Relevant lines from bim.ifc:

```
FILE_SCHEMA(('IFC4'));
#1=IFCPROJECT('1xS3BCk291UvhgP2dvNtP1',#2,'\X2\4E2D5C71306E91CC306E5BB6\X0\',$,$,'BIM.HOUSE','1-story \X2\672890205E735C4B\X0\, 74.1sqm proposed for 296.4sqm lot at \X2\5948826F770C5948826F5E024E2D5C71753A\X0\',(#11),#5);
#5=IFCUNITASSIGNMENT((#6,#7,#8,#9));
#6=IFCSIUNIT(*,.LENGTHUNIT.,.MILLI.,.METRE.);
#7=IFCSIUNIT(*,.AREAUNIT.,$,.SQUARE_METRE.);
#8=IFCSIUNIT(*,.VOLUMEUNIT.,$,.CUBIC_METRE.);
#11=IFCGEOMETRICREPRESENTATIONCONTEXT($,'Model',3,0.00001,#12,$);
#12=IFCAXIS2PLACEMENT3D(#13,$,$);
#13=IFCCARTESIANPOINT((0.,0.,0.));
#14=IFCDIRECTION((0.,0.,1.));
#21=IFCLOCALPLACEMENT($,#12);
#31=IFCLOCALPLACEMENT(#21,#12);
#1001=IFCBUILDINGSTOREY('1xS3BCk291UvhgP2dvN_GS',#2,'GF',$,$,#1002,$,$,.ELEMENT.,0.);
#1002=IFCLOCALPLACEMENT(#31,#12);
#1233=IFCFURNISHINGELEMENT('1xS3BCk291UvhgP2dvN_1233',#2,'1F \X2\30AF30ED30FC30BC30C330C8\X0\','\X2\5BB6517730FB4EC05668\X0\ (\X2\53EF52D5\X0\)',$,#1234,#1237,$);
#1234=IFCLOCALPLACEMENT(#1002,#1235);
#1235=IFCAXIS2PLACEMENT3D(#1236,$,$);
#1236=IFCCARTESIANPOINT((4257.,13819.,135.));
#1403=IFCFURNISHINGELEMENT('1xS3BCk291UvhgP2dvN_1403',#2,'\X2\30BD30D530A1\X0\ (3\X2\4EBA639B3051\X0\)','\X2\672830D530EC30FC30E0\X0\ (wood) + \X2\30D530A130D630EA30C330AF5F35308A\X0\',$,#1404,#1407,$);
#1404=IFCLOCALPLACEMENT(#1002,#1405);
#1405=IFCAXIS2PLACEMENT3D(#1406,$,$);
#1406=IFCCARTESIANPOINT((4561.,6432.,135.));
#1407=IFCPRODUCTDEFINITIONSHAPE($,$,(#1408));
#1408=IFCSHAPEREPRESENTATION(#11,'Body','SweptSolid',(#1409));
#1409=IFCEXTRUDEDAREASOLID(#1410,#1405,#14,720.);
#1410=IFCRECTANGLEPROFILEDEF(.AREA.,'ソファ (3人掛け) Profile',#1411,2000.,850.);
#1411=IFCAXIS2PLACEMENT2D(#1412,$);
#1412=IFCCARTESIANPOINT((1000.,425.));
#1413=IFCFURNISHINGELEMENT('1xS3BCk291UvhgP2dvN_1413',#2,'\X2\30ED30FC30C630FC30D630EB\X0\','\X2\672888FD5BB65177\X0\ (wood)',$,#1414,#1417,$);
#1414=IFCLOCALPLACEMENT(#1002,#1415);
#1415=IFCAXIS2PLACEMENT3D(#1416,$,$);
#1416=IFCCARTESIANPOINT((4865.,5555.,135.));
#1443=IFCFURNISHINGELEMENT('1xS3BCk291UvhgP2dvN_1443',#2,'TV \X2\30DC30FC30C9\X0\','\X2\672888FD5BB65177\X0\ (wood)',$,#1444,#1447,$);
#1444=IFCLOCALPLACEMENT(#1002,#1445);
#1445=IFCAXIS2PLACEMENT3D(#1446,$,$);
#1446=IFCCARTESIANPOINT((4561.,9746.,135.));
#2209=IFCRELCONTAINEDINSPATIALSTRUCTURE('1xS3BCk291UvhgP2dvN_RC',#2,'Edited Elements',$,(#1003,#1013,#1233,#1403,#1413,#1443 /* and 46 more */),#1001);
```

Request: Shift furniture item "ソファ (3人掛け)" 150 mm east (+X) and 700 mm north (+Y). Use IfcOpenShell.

```python
import ifcopenshell
import ifcopenshell.api.geometry
import ifcopenshell.util.placement
import ifcopenshell.util.unit

model = ifcopenshell.open("bim.ifc")
unit_scale = ifcopenshell.util.unit.calculate_unit_scale(model)

item = model.by_guid("1xS3BCk291UvhgP2dvN_1403")
matrix = ifcopenshell.util.placement.get_local_placement(item.ObjectPlacement)
matrix[0, 3] += 0.15 / unit_scale
matrix[1, 3] += 0.7 / unit_scale
ifcopenshell.api.geometry.edit_object_placement(model, product=item, matrix=matrix, is_si=False)

print(ifcopenshell.util.placement.get_local_placement(item.ObjectPlacement).round(3) + 0.0)

model.write("bim_v2.ifc")
```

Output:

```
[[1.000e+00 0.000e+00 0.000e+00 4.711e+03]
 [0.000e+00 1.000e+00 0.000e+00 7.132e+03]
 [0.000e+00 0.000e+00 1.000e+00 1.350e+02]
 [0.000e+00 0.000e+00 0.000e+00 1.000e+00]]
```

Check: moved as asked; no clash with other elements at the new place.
